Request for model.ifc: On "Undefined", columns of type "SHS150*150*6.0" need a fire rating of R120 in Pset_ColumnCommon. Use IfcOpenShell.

First a look at what the model holds.

```python
import ifcopenshell
import ifcopenshell.util.element

model = ifcopenshell.open("model.ifc")
print(model.schema)
storey = next(s for s in model.by_type("IfcBuildingStorey") if s.Name == "Undefined")
columns = [e for e in ifcopenshell.util.element.get_decomposition(storey) if e.is_a("IfcColumn")]
seen = {}
for e in columns:
    element_type = ifcopenshell.util.element.get_type(e)
    key = (element_type.Name if element_type != e and element_type else None, ifcopenshell.util.element.get_pset(e, "Pset_ColumnCommon", "FireRating"))
    seen[key] = seen.get(key, 0) + 1
for (name, value), count in sorted(seen.items(), key=str):
    print(count, "x", name, "|", value)
```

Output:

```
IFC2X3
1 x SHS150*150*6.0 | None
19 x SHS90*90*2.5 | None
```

```python
import ifcopenshell
import ifcopenshell.api.pset
import ifcopenshell.util.element

model = ifcopenshell.open("model.ifc")

storey = next(s for s in model.by_type("IfcBuildingStorey") if s.Name == "Undefined")
columns = [e for e in ifcopenshell.util.element.get_decomposition(storey) if e.is_a("IfcColumn")]

count = 0
for e in columns:
    element_type = ifcopenshell.util.element.get_type(e)
    if element_type in (None, e) or element_type.Name != "SHS150*150*6.0":
        continue
    found = ifcopenshell.util.element.get_pset(e, "Pset_ColumnCommon", should_inherit=False)
    if found:
        pset = model.by_id(found["id"])
        if len(ifcopenshell.util.element.get_elements_by_pset(pset)) > 1:
            pset = ifcopenshell.api.pset.unshare_pset(model, products=[e], pset=pset)[0]
    else:
        pset = ifcopenshell.api.pset.add_pset(model, product=e, name="Pset_ColumnCommon")
    ifcopenshell.api.pset.edit_pset(model, pset=pset, properties={"FireRating": "R120"})
    count += 1

print(count, "columns updated")

model.write("model-out.ifc")
```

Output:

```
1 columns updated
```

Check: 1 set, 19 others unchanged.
